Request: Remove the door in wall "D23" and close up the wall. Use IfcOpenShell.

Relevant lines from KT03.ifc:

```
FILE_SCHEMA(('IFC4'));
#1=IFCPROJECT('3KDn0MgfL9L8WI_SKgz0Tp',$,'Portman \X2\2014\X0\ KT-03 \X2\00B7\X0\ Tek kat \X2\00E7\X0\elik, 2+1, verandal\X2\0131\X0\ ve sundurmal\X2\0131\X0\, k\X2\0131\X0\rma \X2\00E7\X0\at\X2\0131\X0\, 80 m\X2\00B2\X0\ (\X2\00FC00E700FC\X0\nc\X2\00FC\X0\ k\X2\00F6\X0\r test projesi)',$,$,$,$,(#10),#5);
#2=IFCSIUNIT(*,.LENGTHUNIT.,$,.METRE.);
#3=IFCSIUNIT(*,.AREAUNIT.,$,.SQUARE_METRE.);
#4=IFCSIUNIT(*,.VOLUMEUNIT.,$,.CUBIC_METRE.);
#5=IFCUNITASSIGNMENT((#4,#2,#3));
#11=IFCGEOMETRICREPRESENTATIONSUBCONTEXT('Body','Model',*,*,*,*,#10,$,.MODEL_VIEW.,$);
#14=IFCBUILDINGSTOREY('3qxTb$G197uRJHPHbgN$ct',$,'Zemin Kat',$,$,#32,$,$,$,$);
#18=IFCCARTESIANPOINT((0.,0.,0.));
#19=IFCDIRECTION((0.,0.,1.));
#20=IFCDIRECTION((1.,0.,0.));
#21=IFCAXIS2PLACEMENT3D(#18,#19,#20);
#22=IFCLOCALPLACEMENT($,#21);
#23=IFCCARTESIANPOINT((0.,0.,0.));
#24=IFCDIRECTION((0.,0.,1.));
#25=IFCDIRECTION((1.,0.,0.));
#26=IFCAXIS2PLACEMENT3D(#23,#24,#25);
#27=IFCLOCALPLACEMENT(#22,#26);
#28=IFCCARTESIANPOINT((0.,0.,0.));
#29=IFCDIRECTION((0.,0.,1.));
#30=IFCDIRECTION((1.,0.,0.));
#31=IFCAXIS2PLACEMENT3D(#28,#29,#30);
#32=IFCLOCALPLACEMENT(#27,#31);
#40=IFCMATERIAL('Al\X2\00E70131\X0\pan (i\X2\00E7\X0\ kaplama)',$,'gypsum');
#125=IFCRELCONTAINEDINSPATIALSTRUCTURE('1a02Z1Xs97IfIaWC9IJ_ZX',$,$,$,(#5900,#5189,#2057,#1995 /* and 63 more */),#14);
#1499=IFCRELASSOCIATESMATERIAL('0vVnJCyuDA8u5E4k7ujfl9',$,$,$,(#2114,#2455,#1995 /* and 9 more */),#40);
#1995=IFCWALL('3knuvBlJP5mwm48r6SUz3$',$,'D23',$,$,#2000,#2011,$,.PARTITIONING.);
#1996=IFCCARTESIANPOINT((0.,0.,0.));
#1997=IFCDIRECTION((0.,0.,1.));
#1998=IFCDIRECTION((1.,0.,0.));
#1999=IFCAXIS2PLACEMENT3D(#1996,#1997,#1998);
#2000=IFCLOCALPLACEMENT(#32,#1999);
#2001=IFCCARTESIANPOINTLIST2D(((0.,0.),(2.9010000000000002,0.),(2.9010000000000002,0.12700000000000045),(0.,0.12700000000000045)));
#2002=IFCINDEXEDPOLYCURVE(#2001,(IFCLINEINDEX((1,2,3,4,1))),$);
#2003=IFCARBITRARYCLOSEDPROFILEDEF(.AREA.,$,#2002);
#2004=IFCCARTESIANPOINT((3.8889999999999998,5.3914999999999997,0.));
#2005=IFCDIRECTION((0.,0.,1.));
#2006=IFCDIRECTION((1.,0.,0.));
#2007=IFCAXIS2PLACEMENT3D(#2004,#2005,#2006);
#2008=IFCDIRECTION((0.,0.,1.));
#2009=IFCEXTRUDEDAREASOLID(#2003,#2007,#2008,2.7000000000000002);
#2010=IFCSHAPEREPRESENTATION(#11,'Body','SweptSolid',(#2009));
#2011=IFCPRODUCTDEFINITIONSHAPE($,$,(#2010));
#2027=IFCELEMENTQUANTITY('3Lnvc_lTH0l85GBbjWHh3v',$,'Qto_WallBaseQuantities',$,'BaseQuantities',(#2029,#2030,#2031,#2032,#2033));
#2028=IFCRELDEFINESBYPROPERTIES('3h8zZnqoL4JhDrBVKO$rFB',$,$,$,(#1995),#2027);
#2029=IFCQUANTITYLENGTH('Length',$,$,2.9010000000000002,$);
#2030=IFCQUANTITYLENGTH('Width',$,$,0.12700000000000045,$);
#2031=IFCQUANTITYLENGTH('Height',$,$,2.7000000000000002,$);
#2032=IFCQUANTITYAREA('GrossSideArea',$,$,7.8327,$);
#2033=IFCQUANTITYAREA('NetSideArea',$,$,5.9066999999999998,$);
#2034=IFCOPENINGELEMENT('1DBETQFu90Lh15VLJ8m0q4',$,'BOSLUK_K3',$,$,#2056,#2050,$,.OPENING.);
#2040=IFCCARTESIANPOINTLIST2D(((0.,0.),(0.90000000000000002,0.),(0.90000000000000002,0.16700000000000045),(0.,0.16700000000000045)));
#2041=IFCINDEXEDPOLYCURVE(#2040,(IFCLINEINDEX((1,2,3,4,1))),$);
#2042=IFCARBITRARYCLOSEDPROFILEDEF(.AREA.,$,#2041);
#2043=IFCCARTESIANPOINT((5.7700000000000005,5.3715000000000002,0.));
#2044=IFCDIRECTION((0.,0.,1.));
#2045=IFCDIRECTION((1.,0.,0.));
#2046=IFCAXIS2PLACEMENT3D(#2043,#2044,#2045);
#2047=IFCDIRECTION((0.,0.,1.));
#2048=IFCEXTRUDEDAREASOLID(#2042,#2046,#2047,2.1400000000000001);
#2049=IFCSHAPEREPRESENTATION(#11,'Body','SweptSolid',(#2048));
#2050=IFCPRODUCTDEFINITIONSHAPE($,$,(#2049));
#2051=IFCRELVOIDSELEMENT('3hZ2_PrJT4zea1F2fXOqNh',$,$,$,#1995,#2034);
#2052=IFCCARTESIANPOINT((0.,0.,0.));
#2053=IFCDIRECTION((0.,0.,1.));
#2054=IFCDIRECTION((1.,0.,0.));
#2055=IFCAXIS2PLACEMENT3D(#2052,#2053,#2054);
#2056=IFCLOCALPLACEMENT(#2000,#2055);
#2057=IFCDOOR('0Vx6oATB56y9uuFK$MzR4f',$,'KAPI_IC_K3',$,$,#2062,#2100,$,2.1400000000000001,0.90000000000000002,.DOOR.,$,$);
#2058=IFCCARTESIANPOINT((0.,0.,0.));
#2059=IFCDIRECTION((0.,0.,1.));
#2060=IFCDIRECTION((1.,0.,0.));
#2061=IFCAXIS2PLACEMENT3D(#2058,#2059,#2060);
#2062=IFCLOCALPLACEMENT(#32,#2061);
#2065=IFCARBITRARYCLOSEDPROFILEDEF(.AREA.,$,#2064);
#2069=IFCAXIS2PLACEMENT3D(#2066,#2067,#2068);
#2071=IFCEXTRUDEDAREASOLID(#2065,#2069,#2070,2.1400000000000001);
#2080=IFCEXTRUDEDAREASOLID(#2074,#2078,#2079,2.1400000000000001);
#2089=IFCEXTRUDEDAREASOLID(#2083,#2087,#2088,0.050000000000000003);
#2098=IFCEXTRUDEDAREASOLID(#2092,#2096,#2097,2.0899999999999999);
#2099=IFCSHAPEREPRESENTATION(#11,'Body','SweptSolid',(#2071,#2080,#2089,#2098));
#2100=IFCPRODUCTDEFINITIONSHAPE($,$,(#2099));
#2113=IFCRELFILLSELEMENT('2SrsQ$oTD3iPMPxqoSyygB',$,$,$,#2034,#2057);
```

```python
import ifcopenshell
import ifcopenshell.api.feature
import ifcopenshell.api.pset
import ifcopenshell.api.root
import ifcopenshell.geom
import ifcopenshell.util.element
import ifcopenshell.util.shape
import ifcopenshell.util.unit

model = ifcopenshell.open("KT03.ifc")
area_scale = ifcopenshell.util.unit.calculate_unit_scale(model, "AREAUNIT")
settings = ifcopenshell.geom.settings()


def volume(element):
    """Net volume in cubic metres, openings subtracted."""
    shape = ifcopenshell.geom.create_shape(settings, element)
    return ifcopenshell.util.shape.get_volume(shape.geometry)


door = model.by_guid("0Vx6oATB56y9uuFK$MzR4f")
opening = door.FillsVoids[0].RelatingOpeningElement
wall = opening.VoidsElements[0].RelatingBuildingElement
before = volume(wall)

ifcopenshell.api.root.remove_product(model, product=door)
ifcopenshell.api.feature.remove_feature(model, feature=opening)

after = volume(wall)
thickness = 0.127  # wall thickness in metres

# Update the wall's stored quantities.
qto = model.by_id(ifcopenshell.util.element.get_pset(wall, "Qto_WallBaseQuantities", should_inherit=False)["id"])
ifcopenshell.api.pset.edit_qto(model, qto=qto, properties={"NetSideArea": after / thickness / area_scale})

print(f"wall volume {before:.3f} -> {after:.3f} m3")

model.write("KT03-out.ifc")
```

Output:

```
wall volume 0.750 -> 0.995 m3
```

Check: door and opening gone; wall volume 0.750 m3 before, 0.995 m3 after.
